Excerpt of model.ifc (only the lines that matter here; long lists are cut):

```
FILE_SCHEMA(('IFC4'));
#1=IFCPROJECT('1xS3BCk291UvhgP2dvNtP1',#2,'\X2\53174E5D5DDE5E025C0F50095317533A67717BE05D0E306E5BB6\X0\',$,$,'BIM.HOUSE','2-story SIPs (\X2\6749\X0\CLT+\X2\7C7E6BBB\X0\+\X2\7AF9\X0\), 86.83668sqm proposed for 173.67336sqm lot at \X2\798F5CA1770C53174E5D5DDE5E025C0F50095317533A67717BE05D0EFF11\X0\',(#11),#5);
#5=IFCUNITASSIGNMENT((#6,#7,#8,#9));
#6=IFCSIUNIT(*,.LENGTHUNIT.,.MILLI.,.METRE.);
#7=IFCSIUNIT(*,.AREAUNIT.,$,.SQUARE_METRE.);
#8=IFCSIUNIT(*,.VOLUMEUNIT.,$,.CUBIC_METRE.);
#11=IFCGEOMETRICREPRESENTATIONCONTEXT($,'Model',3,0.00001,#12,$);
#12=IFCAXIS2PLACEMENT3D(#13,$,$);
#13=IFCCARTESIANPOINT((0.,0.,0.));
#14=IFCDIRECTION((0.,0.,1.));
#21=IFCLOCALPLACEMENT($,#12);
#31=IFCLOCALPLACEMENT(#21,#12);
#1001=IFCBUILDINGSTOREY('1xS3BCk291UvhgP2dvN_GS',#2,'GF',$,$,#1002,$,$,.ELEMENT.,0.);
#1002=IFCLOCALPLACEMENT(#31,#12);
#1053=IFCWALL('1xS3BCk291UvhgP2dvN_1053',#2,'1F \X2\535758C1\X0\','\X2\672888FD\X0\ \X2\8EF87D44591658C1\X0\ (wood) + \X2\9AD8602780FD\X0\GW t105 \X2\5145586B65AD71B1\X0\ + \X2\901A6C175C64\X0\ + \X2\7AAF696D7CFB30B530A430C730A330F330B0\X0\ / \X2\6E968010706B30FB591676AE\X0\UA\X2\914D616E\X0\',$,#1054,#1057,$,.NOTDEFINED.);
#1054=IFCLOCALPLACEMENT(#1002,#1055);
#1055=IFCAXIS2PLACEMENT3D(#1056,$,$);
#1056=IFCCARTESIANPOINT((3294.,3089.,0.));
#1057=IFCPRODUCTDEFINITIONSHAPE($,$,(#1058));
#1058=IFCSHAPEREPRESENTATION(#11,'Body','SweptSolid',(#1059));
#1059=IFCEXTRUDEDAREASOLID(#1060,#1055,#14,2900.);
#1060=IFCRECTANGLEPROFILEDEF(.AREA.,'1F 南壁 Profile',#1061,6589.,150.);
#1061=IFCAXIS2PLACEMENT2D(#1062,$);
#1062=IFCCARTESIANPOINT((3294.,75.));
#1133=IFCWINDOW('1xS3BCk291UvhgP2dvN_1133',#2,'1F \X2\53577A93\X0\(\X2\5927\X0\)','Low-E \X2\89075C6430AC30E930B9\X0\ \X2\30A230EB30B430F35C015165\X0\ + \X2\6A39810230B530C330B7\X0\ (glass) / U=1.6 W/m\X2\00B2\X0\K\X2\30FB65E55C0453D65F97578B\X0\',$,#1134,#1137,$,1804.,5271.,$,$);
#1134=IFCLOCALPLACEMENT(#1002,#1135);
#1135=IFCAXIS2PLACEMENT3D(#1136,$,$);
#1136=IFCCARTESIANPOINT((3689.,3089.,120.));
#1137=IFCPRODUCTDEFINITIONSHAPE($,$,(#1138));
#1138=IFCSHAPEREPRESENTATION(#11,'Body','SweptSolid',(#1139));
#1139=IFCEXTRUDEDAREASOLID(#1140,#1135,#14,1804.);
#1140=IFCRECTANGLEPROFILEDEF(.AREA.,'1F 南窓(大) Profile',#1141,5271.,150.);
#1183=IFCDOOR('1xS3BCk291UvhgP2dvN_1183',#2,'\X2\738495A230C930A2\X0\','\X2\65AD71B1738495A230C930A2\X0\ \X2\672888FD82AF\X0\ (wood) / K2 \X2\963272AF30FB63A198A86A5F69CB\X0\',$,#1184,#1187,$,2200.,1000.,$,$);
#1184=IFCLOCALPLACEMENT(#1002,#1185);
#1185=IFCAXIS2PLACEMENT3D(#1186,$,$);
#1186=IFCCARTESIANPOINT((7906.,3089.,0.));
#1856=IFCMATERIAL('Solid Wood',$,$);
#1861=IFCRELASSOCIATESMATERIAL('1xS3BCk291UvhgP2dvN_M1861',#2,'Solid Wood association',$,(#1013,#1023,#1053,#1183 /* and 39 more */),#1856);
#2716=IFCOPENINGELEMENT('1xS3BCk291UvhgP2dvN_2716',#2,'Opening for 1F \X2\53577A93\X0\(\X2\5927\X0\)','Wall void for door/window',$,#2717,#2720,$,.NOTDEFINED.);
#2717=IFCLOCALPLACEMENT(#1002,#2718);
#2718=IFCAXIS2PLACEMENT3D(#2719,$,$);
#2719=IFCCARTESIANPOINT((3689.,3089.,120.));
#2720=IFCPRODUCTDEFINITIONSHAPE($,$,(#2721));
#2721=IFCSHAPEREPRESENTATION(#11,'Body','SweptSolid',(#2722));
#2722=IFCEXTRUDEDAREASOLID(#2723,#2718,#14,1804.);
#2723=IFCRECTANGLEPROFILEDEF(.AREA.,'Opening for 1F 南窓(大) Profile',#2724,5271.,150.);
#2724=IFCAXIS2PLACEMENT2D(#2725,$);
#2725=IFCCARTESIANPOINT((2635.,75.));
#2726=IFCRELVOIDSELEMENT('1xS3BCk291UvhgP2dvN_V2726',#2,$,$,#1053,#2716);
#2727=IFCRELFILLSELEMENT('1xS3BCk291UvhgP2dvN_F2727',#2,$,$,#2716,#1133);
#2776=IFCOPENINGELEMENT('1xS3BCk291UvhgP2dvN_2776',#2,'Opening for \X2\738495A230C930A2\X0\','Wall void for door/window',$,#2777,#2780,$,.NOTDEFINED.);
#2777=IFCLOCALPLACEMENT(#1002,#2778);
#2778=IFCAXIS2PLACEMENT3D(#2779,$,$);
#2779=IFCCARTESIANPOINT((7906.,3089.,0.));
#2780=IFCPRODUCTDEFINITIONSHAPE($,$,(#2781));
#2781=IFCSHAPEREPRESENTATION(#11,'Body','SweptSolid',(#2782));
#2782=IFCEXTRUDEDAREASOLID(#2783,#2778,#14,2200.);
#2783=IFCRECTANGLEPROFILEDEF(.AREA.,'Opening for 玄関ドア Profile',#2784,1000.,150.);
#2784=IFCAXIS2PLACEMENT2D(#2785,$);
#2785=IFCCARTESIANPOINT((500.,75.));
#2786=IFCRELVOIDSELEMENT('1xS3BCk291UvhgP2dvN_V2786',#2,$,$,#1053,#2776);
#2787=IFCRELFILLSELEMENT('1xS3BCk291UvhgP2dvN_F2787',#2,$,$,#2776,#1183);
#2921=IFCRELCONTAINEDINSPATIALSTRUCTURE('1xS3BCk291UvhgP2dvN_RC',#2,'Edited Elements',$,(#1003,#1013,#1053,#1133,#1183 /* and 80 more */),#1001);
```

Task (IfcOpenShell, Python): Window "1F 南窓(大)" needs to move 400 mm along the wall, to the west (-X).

```python
import ifcopenshell
import ifcopenshell.api.geometry
import ifcopenshell.util.placement
import ifcopenshell.util.unit

model = ifcopenshell.open("model.ifc")
unit_scale = ifcopenshell.util.unit.calculate_unit_scale(model)

window = model.by_guid("1xS3BCk291UvhgP2dvN_1133")
opening = window.FillsVoids[0].RelatingOpeningElement
wall = opening.VoidsElements[0].RelatingBuildingElement

wall_matrix = ifcopenshell.util.placement.get_local_placement(wall.ObjectPlacement)
shift = wall_matrix[:3, 0] * -0.4 / unit_scale
before = ifcopenshell.util.placement.get_local_placement(window.ObjectPlacement)[:3, 3].copy()

# The window is not placed relative to its opening, so move both.
for product in (opening, window):
    matrix = ifcopenshell.util.placement.get_local_placement(product.ObjectPlacement)
    matrix[:3, 3] += shift
    ifcopenshell.api.geometry.edit_object_placement(model, product=product, matrix=matrix, is_si=False)

after = ifcopenshell.util.placement.get_local_placement(window.ObjectPlacement)[:3, 3]
print("window moved by", (after - before).round(3) + 0.0)

model.write("model-out.ifc")
```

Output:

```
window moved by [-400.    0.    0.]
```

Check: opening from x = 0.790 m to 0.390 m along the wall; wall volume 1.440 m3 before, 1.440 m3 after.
